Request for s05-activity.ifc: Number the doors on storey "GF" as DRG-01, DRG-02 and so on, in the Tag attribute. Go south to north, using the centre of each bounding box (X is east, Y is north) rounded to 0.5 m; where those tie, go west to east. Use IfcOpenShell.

First a look at what the model holds.

```python
import ifcopenshell
import ifcopenshell.util.element
import ifcopenshell.util.placement

model = ifcopenshell.open("s05-activity.ifc")
print(model.schema)
storey = next(s for s in model.by_type("IfcBuildingStorey") if s.Name == "GF")
doors = [e for e in ifcopenshell.util.element.get_decomposition(storey) if e.is_a("IfcDoor")]
for e in sorted(doors, key=lambda e: e.id()):
    origin = ifcopenshell.util.placement.get_local_placement(e.ObjectPlacement)[:3, 3]
    print(e.id(), e.Tag, e.Name, origin.round(2) + 0.0, sep=" | ")
```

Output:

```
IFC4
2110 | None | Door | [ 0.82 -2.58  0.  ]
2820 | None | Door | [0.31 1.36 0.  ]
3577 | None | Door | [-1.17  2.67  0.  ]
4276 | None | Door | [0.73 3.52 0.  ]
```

```python
import ifcopenshell
import ifcopenshell.geom
import ifcopenshell.util.element
import ifcopenshell.util.shape

model = ifcopenshell.open("s05-activity.ifc")
settings = ifcopenshell.geom.settings()
settings.set("use-world-coords", True)


def centre(element):
    shape = ifcopenshell.geom.create_shape(settings, element)
    return ifcopenshell.util.shape.get_bbox_centroid(shape.geometry)


storey = next(s for s in model.by_type("IfcBuildingStorey") if s.Name == "GF")
doors = [e for e in ifcopenshell.util.element.get_decomposition(storey) if e.is_a("IfcDoor")]

# Insertion points can sit at a corner or the storey origin, so sort by the geometry (in metres).
centres = {e: centre(e) for e in doors}
doors.sort(key=lambda e: (round(centres[e][1] / 0.5), centres[e][0]))

for i, e in enumerate(doors, start=1):
    number = f"DRG-{i:02d}"
    e.Tag = number
    print(e.id(), number)

model.write("s05-activity_rev.ifc")
```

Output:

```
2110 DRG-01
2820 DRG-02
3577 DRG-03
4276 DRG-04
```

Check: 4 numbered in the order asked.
